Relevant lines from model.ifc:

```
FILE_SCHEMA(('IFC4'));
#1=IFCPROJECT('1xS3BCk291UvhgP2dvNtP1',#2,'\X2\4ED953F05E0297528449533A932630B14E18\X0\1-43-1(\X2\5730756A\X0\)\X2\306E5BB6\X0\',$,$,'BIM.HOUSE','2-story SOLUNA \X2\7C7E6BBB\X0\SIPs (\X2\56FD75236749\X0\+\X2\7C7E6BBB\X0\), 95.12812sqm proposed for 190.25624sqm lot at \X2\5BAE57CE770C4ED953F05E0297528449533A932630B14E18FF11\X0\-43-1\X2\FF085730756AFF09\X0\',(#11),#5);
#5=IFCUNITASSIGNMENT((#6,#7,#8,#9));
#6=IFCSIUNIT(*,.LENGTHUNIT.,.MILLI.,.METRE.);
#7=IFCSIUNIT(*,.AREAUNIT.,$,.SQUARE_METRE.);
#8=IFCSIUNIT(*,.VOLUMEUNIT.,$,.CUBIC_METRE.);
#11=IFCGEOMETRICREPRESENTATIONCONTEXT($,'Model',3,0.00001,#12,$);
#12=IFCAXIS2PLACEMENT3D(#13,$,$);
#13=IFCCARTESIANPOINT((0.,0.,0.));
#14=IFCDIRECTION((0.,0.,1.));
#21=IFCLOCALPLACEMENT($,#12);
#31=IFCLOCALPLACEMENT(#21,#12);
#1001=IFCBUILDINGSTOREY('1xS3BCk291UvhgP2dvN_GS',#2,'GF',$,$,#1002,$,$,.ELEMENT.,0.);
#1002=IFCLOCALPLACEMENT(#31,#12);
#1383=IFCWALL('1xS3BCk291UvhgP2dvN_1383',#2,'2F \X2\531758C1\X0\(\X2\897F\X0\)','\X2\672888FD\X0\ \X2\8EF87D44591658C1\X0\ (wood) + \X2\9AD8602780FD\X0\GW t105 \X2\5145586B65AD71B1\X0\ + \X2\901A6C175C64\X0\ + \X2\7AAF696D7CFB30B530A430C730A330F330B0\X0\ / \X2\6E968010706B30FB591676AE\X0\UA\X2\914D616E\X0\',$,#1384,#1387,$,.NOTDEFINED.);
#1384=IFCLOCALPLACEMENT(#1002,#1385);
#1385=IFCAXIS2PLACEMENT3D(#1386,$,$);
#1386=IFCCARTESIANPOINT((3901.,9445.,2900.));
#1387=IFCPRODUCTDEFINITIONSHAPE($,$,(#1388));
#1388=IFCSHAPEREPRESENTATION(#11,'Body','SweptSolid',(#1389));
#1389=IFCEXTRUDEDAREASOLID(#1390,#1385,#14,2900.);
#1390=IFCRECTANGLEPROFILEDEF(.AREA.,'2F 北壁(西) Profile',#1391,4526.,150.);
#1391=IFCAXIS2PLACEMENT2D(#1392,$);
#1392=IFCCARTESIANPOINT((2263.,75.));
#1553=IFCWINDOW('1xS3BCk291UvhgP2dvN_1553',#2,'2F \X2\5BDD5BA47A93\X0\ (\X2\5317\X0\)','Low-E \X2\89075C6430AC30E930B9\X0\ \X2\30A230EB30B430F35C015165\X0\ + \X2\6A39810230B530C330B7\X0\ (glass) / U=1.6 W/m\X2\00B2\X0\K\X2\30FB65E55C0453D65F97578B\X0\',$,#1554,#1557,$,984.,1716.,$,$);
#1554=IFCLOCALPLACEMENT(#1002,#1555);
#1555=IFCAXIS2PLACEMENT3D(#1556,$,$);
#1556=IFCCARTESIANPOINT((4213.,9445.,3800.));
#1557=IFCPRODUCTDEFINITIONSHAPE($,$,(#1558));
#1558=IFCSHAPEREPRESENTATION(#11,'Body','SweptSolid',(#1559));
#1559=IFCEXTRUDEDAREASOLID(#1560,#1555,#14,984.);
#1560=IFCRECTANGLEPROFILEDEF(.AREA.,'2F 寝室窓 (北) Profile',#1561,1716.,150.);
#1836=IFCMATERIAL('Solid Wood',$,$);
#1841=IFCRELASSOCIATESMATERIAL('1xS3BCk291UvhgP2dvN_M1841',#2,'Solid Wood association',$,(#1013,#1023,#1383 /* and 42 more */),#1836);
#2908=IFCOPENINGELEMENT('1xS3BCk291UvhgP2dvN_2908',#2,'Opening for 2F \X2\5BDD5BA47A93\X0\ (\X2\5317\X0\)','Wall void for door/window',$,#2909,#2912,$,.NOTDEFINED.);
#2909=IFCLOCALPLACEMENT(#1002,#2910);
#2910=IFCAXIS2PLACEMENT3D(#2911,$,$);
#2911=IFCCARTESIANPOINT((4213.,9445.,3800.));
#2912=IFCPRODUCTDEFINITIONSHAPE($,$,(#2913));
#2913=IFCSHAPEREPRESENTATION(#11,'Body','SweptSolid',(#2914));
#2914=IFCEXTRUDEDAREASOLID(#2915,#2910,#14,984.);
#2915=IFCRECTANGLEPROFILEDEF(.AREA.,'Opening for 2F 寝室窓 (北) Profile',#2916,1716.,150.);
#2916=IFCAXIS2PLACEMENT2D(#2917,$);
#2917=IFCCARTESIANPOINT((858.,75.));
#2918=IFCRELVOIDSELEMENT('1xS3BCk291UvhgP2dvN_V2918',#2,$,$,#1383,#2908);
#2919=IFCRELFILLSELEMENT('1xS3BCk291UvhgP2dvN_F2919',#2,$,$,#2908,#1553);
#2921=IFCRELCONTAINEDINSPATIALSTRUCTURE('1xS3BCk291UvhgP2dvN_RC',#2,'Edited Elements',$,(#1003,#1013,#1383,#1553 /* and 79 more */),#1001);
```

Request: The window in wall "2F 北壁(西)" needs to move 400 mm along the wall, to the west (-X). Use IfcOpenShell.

```python
import ifcopenshell
import ifcopenshell.api.geometry
import ifcopenshell.util.placement
import ifcopenshell.util.unit

model = ifcopenshell.open("model.ifc")
unit_scale = ifcopenshell.util.unit.calculate_unit_scale(model)

window = model.by_id(1553)
opening = window.FillsVoids[0].RelatingOpeningElement
wall = opening.VoidsElements[0].RelatingBuildingElement

wall_matrix = ifcopenshell.util.placement.get_local_placement(wall.ObjectPlacement)
shift = wall_matrix[:3, 0] * -0.4 / unit_scale
before = ifcopenshell.util.placement.get_local_placement(window.ObjectPlacement)[:3, 3].copy()

# The window is not placed relative to its opening, so move both.
for product in (opening, window):
    matrix = ifcopenshell.util.placement.get_local_placement(product.ObjectPlacement)
    matrix[:3, 3] += shift
    ifcopenshell.api.geometry.edit_object_placement(model, product=product, matrix=matrix, is_si=False)

after = ifcopenshell.util.placement.get_local_placement(window.ObjectPlacement)[:3, 3]
print("window moved by", (after - before).round(3) + 0.0)

model.write("model_updated.ifc")
```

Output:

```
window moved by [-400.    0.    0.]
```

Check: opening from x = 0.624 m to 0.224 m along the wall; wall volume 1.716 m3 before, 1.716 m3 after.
